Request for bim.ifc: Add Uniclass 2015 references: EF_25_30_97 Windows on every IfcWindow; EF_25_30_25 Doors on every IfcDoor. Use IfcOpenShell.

First a look at what the model holds.

```python
import ifcopenshell

model = ifcopenshell.open("bim.ifc")
print(model.schema)
print("classifications:", [c.Name for c in model.by_type("IfcClassification")])
for ifc_class in ("IfcDoor", "IfcRoof", "IfcStair", "IfcWall", "IfcWindow"):
    print(ifc_class, len(model.by_type(ifc_class)))
```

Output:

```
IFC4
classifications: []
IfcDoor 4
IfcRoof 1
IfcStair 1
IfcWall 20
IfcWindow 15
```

```python
import ifcopenshell
import ifcopenshell.api.classification

model = ifcopenshell.open("bim.ifc")

system = ifcopenshell.api.classification.add_classification(model, classification="Uniclass 2015")

codes = {
    "IfcWindow": ("EF_25_30_97", "Windows"),
    "IfcDoor": ("EF_25_30_25", "Doors"),
}
for ifc_class, (code, name) in codes.items():
    products = model.by_type(ifc_class)
    ifcopenshell.api.classification.add_reference(
        model, products=products, classification=system, identification=code, name=name
    )
    print(code, len(products))

model.write("bim-out.ifc")
```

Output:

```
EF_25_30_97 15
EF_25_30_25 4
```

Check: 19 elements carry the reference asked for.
